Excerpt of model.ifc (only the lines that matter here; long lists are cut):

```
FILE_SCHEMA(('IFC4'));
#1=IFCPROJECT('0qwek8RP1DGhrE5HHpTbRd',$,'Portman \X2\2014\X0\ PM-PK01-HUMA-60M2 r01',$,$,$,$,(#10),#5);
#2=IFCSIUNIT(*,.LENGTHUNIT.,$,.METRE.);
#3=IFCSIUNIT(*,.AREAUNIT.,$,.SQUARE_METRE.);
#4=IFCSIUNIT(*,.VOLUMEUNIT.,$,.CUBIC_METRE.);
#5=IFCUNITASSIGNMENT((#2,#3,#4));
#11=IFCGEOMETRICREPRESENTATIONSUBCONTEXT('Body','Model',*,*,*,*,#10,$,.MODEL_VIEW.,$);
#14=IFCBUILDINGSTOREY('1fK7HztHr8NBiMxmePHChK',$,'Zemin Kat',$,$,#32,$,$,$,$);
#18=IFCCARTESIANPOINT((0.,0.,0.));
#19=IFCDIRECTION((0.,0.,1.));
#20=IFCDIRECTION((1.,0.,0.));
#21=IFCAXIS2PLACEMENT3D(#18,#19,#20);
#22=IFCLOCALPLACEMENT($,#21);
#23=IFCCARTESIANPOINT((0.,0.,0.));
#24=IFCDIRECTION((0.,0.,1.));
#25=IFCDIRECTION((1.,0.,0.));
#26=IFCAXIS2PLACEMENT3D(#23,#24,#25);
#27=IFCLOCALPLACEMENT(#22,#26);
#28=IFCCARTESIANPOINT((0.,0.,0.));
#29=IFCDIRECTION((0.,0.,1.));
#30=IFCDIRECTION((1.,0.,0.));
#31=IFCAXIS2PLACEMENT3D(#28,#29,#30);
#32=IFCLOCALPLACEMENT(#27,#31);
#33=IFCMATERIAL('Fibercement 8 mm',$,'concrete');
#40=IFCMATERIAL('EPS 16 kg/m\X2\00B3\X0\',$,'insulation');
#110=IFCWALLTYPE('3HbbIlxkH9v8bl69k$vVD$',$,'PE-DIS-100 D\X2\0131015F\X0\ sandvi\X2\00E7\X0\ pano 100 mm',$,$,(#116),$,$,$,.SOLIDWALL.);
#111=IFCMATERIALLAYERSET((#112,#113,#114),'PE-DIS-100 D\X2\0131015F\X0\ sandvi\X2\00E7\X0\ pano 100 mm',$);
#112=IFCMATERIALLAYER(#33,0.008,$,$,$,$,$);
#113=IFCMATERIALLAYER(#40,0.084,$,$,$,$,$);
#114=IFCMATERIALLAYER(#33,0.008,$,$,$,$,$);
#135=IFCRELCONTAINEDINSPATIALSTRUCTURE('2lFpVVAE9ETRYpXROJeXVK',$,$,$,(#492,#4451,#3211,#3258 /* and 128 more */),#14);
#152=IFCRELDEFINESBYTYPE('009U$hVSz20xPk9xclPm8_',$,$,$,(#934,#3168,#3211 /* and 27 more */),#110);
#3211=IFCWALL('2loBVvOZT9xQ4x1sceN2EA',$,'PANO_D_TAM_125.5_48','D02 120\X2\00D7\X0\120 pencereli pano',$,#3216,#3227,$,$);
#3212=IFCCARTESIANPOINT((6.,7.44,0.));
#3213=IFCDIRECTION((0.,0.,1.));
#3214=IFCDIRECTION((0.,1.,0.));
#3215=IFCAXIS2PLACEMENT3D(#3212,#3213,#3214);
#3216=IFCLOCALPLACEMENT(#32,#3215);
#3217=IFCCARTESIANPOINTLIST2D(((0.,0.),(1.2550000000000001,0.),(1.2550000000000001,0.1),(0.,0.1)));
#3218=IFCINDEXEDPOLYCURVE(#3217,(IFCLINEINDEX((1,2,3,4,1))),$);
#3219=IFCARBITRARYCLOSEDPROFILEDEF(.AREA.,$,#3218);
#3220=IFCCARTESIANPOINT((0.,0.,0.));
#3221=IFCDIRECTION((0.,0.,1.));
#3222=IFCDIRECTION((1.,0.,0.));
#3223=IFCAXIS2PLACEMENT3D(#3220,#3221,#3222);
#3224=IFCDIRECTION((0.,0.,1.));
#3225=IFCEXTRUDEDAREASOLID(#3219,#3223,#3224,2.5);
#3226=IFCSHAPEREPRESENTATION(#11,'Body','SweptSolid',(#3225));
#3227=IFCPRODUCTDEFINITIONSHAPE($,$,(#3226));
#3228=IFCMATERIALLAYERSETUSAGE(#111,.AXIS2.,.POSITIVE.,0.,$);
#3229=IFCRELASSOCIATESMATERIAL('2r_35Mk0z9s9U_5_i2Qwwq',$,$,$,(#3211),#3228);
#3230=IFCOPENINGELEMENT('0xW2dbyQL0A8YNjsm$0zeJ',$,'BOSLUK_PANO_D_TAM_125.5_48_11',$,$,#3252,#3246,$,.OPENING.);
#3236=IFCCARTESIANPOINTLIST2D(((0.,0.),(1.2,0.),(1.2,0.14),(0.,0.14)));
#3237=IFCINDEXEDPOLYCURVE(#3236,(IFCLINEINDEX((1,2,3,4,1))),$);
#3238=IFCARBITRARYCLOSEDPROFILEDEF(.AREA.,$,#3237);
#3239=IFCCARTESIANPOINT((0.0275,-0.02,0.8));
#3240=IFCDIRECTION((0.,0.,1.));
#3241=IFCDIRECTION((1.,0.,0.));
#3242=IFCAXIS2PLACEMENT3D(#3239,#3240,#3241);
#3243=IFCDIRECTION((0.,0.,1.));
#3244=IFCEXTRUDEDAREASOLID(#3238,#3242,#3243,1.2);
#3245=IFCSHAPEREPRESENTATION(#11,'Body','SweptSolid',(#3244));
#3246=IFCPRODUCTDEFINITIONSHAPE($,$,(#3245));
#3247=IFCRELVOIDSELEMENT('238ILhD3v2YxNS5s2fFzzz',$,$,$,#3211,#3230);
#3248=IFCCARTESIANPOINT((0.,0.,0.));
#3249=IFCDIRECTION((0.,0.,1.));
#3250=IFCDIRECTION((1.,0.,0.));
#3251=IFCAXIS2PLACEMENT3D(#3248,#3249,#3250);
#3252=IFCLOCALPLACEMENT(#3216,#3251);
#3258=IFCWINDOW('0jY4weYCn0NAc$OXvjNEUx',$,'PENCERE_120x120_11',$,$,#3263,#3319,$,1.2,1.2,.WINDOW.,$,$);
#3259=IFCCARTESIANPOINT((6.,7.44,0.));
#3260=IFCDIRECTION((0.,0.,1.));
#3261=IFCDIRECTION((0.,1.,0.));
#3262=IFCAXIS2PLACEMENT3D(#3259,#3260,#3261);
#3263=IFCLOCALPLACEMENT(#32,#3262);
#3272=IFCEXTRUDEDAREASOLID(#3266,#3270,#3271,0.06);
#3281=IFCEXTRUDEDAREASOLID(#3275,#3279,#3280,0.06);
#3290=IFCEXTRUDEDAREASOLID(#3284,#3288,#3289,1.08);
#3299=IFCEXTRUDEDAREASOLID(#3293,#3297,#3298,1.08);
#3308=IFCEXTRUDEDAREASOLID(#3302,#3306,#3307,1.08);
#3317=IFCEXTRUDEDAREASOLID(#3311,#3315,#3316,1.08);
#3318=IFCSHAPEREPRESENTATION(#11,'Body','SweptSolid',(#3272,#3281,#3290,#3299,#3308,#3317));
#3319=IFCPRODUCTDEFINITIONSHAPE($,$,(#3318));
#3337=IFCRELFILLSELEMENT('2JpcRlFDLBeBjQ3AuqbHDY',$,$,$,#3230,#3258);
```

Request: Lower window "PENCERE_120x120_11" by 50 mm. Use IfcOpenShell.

```python
import numpy as np
import ifcopenshell
import ifcopenshell.api.geometry
import ifcopenshell.util.placement
import ifcopenshell.util.unit

model = ifcopenshell.open("model.ifc")
unit_scale = ifcopenshell.util.unit.calculate_unit_scale(model)

window = model.by_guid("0jY4weYCn0NAc$OXvjNEUx")
opening = window.FillsVoids[0].RelatingOpeningElement
dz = -0.05 / unit_scale

shift = np.array([0.0, 0.0, dz])
# The window is not placed relative to its opening, so move both.
for product in (opening, window):
    matrix = ifcopenshell.util.placement.get_local_placement(product.ObjectPlacement)
    matrix[:3, 3] += shift
    ifcopenshell.api.geometry.edit_object_placement(model, product=product, matrix=matrix, is_si=False)

print(f"moved by {dz * unit_scale:+.3f} m")

model.write("model_updated.ifc")
```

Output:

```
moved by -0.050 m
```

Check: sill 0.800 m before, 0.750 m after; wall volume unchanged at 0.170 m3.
